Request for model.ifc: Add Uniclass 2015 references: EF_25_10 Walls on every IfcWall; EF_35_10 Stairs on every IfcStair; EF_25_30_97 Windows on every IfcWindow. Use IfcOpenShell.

First a look at what the model holds.

```python
import ifcopenshell

model = ifcopenshell.open("model.ifc")
print(model.schema)
print("classifications:", [c.Name for c in model.by_type("IfcClassification")])
for ifc_class in ("IfcDoor", "IfcRoof", "IfcStair", "IfcWall", "IfcWindow"):
    print(ifc_class, len(model.by_type(ifc_class)))
```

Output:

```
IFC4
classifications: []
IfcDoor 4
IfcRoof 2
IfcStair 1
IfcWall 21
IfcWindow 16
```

```python
import ifcopenshell
import ifcopenshell.api.classification

model = ifcopenshell.open("model.ifc")

system = ifcopenshell.api.classification.add_classification(model, classification="Uniclass 2015")

codes = {
    "IfcWall": ("EF_25_10", "Walls"),
    "IfcStair": ("EF_35_10", "Stairs"),
    "IfcWindow": ("EF_25_30_97", "Windows"),
}
for ifc_class, (code, name) in codes.items():
    products = model.by_type(ifc_class)
    ifcopenshell.api.classification.add_reference(
        model, products=products, classification=system, identification=code, name=name
    )
    print(code, len(products))

model.write("model_updated.ifc")
```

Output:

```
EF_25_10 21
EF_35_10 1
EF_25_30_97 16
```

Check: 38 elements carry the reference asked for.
